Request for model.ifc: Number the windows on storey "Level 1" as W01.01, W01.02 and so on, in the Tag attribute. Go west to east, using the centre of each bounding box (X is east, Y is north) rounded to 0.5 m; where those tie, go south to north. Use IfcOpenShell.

First a look at what the model holds.

```python
import ifcopenshell
import ifcopenshell.util.element
import ifcopenshell.util.placement

model = ifcopenshell.open("model.ifc")
print(model.schema)
storey = next(s for s in model.by_type("IfcBuildingStorey") if s.Name == "Level 1")
windows = [e for e in ifcopenshell.util.element.get_decomposition(storey) if e.is_a("IfcWindow")]
for e in sorted(windows, key=lambda e: e.id()):
    origin = ifcopenshell.util.placement.get_local_placement(e.ObjectPlacement)[:3, 3]
    print(e.id(), e.Tag, e.Name, origin.round(2) + 0.0, sep=" | ")
```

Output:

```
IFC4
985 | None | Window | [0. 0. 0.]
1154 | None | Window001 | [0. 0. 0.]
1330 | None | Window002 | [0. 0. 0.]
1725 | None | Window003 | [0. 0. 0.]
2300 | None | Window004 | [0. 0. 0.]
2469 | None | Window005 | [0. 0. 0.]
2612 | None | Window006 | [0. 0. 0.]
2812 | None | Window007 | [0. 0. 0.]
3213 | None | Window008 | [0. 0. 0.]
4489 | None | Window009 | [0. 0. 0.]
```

```python
import ifcopenshell
import ifcopenshell.geom
import ifcopenshell.util.element
import ifcopenshell.util.shape

model = ifcopenshell.open("model.ifc")
settings = ifcopenshell.geom.settings()
settings.set("use-world-coords", True)


def centre(element):
    shape = ifcopenshell.geom.create_shape(settings, element)
    return ifcopenshell.util.shape.get_bbox_centroid(shape.geometry)


storey = next(s for s in model.by_type("IfcBuildingStorey") if s.Name == "Level 1")
windows = [e for e in ifcopenshell.util.element.get_decomposition(storey) if e.is_a("IfcWindow")]

# Insertion points can sit at a corner or the storey origin, so sort by the geometry (in metres).
centres = {e: centre(e) for e in windows}
windows.sort(key=lambda e: (round(centres[e][0] / 0.5), centres[e][1]))

for i, e in enumerate(windows, start=1):
    number = f"W01.{i:02d}"
    e.Tag = number
    print(e.id(), number)

model.write("model_updated.ifc")
```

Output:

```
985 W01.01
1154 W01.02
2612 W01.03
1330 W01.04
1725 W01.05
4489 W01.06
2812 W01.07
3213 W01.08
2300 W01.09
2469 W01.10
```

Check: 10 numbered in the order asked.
